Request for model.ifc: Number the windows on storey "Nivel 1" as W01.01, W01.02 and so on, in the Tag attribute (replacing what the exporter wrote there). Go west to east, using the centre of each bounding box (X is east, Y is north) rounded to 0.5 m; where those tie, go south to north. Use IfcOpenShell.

First a look at what the model holds.

```python
import ifcopenshell
import ifcopenshell.util.element
import ifcopenshell.util.placement

model = ifcopenshell.open("model.ifc")
print(model.schema)
storey = next(s for s in model.by_type("IfcBuildingStorey") if s.Name == "Nivel 1")
windows = [e for e in ifcopenshell.util.element.get_decomposition(storey) if e.is_a("IfcWindow")]
for e in sorted(windows, key=lambda e: e.id()):
    origin = ifcopenshell.util.placement.get_local_placement(e.ObjectPlacement)[:3, 3]
    print(e.id(), e.Tag, e.Name, origin.round(2) + 0.0, sep=" | ")
```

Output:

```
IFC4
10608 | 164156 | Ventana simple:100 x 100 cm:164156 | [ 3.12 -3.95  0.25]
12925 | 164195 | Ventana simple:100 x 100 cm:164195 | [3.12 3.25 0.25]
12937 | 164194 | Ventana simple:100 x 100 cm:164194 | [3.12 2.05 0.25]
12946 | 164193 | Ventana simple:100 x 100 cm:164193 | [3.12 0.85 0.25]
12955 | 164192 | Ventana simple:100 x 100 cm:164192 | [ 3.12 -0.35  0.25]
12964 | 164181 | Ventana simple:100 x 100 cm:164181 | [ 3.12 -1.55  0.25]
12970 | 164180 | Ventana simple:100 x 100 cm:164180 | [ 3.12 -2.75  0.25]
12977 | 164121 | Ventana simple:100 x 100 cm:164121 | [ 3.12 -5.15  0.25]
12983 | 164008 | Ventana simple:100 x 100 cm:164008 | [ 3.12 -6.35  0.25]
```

```python
import ifcopenshell
import ifcopenshell.geom
import ifcopenshell.util.element
import ifcopenshell.util.shape

model = ifcopenshell.open("model.ifc")
settings = ifcopenshell.geom.settings()
settings.set("use-world-coords", True)


def centre(element):
    shape = ifcopenshell.geom.create_shape(settings, element)
    return ifcopenshell.util.shape.get_bbox_centroid(shape.geometry)


storey = next(s for s in model.by_type("IfcBuildingStorey") if s.Name == "Nivel 1")
windows = [e for e in ifcopenshell.util.element.get_decomposition(storey) if e.is_a("IfcWindow")]

# Insertion points can sit at a corner or the storey origin, so sort by the geometry (in metres).
centres = {e: centre(e) for e in windows}
windows.sort(key=lambda e: (round(centres[e][0] / 0.5), centres[e][1]))

for i, e in enumerate(windows, start=1):
    number = f"W01.{i:02d}"
    e.Tag = number
    print(e.id(), number)

model.write("model-out.ifc")
```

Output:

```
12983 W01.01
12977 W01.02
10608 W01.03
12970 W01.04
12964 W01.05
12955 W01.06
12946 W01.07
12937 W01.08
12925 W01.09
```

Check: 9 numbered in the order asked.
